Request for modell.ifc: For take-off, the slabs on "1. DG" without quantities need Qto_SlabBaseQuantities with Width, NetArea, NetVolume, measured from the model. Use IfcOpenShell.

First a look at what the model holds.

```python
import ifcopenshell
import ifcopenshell.util.element
import ifcopenshell.util.unit

model = ifcopenshell.open("modell.ifc")
print(model.schema)
for unit_type in ("LENGTHUNIT", "AREAUNIT", "VOLUMEUNIT"):
    print(unit_type, ifcopenshell.util.unit.calculate_unit_scale(model, unit_type))
storey = next(s for s in model.by_type("IfcBuildingStorey") if s.Name == "1. DG")
slabs = [e for e in ifcopenshell.util.element.get_decomposition(storey) if e.is_a("IfcSlab")]
for e in sorted(slabs, key=lambda e: e.id()):
    print(e.id(), e.is_a(), e.Name, list(ifcopenshell.util.element.get_psets(e, qtos_only=True)), sep=" | ")
```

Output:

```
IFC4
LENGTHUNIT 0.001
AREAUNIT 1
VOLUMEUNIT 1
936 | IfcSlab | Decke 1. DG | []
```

```python
import ifcopenshell
import ifcopenshell.api.pset
import ifcopenshell.geom
import ifcopenshell.util.element
import ifcopenshell.util.shape
import ifcopenshell.util.unit

model = ifcopenshell.open("modell.ifc")
unit_scale = ifcopenshell.util.unit.calculate_unit_scale(model)
area_scale = ifcopenshell.util.unit.calculate_unit_scale(model, "AREAUNIT")
volume_scale = ifcopenshell.util.unit.calculate_unit_scale(model, "VOLUMEUNIT")
settings = ifcopenshell.geom.settings()

storey = next(s for s in model.by_type("IfcBuildingStorey") if s.Name == "1. DG")
slabs = [e for e in ifcopenshell.util.element.get_decomposition(storey) if e.is_a("IfcSlab")]

for e in sorted(slabs, key=lambda e: e.id()):
    if ifcopenshell.util.element.get_psets(e, qtos_only=True, should_inherit=False):
        continue
    # Geometry comes back in metres, in the element's own axes.
    shape = ifcopenshell.geom.create_shape(settings, e)
    values = {
        "Width": ifcopenshell.util.shape.get_z(shape.geometry) / unit_scale,
        "NetArea": ifcopenshell.util.shape.get_footprint_area(shape.geometry) / area_scale,
        "NetVolume": ifcopenshell.util.shape.get_volume(shape.geometry) / volume_scale,
    }
    qto = ifcopenshell.api.pset.add_qto(model, product=e, name="Qto_SlabBaseQuantities")
    ifcopenshell.api.pset.edit_qto(model, qto=qto, properties=values)
    print(e.id(), {k: round(v, 3) for k, v in values.items()})

model.write("modell-out.ifc")
```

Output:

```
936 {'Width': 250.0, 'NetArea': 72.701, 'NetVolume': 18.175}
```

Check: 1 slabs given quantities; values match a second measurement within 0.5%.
